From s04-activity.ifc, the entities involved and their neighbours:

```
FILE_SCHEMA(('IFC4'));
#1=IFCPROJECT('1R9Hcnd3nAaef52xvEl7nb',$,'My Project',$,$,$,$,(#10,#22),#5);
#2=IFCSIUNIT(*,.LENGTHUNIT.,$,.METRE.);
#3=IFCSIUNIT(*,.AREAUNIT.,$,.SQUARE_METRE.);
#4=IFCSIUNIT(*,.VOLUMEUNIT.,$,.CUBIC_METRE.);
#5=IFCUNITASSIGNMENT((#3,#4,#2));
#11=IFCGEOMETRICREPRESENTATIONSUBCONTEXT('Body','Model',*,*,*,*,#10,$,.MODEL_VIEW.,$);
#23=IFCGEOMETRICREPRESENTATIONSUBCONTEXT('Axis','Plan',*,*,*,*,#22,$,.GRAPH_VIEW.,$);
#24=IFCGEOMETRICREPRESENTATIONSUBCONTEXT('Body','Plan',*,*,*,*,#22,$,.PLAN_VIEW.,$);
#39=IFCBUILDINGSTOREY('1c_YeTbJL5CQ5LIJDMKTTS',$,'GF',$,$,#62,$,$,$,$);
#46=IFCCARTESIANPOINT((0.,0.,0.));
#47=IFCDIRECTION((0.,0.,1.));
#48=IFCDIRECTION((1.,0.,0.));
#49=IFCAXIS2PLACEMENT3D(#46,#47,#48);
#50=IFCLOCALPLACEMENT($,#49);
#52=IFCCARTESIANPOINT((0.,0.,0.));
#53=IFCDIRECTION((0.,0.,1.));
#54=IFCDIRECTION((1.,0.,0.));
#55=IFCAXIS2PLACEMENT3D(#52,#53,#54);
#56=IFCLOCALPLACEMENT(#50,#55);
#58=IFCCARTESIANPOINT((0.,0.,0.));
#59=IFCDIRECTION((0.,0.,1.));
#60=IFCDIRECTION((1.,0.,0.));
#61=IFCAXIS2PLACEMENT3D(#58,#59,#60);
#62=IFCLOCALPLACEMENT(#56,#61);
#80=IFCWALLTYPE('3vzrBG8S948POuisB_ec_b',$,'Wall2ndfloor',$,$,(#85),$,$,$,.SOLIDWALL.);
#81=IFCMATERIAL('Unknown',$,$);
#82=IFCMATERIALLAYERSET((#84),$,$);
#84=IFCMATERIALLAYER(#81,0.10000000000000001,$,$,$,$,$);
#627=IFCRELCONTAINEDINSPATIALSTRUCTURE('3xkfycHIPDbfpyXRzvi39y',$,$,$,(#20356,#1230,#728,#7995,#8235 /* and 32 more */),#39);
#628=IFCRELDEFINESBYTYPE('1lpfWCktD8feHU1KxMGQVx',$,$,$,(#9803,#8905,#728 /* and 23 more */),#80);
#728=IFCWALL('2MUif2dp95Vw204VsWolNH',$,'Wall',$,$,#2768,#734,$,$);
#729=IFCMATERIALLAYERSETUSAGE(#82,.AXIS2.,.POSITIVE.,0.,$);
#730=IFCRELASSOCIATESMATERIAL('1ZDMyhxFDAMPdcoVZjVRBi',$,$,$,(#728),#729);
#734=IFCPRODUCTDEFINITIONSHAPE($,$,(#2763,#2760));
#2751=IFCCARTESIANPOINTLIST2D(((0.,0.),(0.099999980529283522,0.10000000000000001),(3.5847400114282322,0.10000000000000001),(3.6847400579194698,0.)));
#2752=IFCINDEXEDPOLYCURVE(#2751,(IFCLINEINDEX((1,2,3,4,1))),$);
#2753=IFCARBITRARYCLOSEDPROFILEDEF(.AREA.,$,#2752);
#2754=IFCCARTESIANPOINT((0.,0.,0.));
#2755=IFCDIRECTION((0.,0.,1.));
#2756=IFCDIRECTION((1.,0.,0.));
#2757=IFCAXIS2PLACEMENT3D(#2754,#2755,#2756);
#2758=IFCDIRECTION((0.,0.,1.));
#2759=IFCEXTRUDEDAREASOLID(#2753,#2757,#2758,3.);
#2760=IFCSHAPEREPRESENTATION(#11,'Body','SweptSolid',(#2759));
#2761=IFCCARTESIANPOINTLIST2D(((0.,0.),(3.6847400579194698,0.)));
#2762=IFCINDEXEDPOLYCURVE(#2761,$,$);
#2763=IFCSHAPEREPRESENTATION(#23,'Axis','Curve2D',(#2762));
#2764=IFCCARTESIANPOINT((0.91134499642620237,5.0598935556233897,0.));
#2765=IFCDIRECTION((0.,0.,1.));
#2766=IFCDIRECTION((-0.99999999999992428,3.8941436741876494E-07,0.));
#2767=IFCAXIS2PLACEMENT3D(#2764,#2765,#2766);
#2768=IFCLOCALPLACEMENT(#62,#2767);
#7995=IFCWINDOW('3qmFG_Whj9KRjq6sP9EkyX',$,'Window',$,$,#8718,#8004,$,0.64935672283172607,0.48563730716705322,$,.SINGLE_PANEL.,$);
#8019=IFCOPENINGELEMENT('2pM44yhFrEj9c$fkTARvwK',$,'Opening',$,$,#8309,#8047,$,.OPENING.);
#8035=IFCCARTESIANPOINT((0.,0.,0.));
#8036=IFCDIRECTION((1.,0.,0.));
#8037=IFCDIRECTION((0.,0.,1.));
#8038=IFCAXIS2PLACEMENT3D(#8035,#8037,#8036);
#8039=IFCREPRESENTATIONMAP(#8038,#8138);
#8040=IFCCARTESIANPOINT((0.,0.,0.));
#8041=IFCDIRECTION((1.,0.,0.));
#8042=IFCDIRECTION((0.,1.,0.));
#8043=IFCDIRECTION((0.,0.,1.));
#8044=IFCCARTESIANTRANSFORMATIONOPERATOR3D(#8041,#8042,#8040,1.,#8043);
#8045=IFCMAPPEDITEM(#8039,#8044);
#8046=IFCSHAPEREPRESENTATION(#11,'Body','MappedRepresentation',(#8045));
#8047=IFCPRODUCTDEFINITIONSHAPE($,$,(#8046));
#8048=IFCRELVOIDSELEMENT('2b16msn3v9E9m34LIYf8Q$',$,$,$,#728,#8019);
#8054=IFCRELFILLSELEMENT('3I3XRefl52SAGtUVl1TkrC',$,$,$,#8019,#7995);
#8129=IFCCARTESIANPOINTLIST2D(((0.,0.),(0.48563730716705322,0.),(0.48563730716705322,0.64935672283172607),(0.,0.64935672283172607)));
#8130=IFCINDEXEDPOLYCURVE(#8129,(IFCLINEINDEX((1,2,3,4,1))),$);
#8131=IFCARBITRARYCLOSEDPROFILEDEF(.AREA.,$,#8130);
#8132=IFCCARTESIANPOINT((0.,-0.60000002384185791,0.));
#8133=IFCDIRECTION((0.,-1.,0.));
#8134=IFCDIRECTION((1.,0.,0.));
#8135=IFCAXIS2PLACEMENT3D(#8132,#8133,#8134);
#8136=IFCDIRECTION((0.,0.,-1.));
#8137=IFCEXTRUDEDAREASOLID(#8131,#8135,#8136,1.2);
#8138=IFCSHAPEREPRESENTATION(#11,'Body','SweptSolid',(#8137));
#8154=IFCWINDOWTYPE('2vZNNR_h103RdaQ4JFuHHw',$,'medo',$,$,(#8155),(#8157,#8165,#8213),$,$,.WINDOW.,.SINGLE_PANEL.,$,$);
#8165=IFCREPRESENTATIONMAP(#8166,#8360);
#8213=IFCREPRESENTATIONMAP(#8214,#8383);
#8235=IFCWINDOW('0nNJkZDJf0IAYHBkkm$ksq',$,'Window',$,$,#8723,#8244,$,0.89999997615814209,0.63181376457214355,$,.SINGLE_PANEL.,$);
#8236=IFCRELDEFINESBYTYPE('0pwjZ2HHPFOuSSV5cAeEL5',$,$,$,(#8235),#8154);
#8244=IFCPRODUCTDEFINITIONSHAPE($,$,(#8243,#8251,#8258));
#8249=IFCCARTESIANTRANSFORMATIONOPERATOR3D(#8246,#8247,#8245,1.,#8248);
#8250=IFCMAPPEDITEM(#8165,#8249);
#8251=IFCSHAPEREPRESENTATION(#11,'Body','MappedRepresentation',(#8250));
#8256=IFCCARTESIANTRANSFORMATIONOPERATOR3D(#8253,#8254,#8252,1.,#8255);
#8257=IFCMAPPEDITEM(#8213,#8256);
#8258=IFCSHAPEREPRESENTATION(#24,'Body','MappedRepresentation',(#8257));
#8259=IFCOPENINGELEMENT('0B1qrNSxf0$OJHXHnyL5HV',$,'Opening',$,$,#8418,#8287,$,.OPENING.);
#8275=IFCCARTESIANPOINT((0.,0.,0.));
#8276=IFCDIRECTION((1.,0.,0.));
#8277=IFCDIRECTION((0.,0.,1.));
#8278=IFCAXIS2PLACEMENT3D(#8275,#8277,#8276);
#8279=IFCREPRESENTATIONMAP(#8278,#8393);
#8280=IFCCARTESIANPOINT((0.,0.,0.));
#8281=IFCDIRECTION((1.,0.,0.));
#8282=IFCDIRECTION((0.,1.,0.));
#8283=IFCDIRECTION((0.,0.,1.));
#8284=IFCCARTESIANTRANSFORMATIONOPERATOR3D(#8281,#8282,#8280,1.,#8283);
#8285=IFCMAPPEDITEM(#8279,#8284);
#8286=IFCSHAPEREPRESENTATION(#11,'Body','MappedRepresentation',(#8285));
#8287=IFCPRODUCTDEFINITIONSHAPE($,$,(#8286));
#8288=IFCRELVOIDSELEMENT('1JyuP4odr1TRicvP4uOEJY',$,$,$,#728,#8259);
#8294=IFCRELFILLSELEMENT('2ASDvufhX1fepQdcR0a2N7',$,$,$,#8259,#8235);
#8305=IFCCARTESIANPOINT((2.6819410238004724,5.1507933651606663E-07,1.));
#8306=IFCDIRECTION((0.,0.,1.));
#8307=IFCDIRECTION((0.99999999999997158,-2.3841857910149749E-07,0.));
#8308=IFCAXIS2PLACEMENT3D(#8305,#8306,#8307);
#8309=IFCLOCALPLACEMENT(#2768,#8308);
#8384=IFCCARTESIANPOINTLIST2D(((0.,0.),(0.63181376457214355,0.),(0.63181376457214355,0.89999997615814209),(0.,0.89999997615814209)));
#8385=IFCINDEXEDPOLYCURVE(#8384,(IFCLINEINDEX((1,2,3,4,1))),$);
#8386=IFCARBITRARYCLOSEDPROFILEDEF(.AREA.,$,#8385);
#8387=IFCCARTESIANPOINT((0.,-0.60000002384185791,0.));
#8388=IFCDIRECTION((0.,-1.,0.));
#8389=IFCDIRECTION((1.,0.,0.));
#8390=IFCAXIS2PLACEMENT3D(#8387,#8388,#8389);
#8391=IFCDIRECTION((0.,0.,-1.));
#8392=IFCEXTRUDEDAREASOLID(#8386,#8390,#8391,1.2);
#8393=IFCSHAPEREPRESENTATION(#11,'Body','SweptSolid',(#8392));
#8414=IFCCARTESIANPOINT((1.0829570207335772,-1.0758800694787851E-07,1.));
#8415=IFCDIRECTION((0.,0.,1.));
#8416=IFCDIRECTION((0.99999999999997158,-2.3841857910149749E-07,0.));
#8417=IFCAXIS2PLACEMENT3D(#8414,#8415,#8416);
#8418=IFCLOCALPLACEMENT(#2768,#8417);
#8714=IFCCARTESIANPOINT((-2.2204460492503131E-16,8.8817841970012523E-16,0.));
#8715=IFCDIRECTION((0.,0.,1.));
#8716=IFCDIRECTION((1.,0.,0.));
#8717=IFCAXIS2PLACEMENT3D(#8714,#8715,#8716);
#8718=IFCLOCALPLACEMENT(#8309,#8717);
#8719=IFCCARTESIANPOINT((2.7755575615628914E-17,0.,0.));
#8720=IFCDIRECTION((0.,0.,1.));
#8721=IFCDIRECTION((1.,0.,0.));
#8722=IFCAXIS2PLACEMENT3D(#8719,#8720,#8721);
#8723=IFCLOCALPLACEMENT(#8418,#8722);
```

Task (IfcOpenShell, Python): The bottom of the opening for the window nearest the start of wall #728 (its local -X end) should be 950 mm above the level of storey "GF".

```python
import numpy as np
import ifcopenshell
import ifcopenshell.api.geometry
import ifcopenshell.geom
import ifcopenshell.util.element
import ifcopenshell.util.placement
import ifcopenshell.util.shape
import ifcopenshell.util.unit

model = ifcopenshell.open("s04-activity.ifc")
unit_scale = ifcopenshell.util.unit.calculate_unit_scale(model)

window = model.by_id(8235)
opening = window.FillsVoids[0].RelatingOpeningElement
storey = ifcopenshell.util.element.get_container(window, ifc_class="IfcBuildingStorey")
level = ifcopenshell.util.placement.get_local_placement(storey.ObjectPlacement)[2, 3]

# The opening's origin need not be at the sill, so measure its lowest point.
shape = ifcopenshell.geom.create_shape(ifcopenshell.geom.settings(), opening)
bottom = ifcopenshell.util.shape.get_shape_bottom_elevation(shape, shape.geometry) / unit_scale
dz = level + 0.95 - bottom

shift = np.array([0.0, 0.0, dz])
# The window is placed relative to its opening, so it follows when the opening moves.
matrix = ifcopenshell.util.placement.get_local_placement(opening.ObjectPlacement)
matrix[:3, 3] += shift
ifcopenshell.api.geometry.edit_object_placement(
    model, product=opening, matrix=matrix, is_si=False, should_transform_children=True
)

print(f"moved by {dz * unit_scale:+.3f} m")

model.write("s04-activity_updated.ifc")
```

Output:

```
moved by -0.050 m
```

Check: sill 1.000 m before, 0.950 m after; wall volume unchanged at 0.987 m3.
